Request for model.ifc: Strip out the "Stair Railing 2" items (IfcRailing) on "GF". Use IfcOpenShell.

First a look at what the model holds.

```python
import ifcopenshell
import ifcopenshell.util.element

model = ifcopenshell.open("model.ifc")
print(model.schema)
storey = next(s for s in model.by_type("IfcBuildingStorey") if s.Name == "GF")
railings = [e for e in ifcopenshell.util.element.get_decomposition(storey) if e.is_a("IfcRailing")]
seen = {}
for e in railings:
    element_type = ifcopenshell.util.element.get_type(e)
    name = element_type.Name if element_type not in (None, e) else None
    seen[name] = seen.get(name, 0) + 1
for name, count in sorted(seen.items(), key=str):
    print(count, "x", name)
```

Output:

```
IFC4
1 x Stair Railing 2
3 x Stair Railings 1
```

```python
import ifcopenshell
import ifcopenshell.api.root
import ifcopenshell.util.element

model = ifcopenshell.open("model.ifc")

storey = next(s for s in model.by_type("IfcBuildingStorey") if s.Name == "GF")
railings = [e for e in ifcopenshell.util.element.get_decomposition(storey) if e.is_a("IfcRailing")]
targets = [e for e in railings if (t := ifcopenshell.util.element.get_type(e)) not in (None, e) and t.Name == "Stair Railing 2"]

for e in targets:
    ifcopenshell.api.root.remove_product(model, product=e)
print(len(targets), "removed")

model.write("model-out.ifc")
```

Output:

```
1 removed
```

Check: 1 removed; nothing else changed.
